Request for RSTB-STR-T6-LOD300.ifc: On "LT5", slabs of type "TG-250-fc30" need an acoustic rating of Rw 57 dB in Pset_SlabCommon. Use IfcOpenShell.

First a look at what the model holds.

```python
import ifcopenshell
import ifcopenshell.util.element

model = ifcopenshell.open("RSTB-STR-T6-LOD300.ifc")
print(model.schema)
storey = next(s for s in model.by_type("IfcBuildingStorey") if s.Name == "LT5")
slabs = [e for e in ifcopenshell.util.element.get_decomposition(storey) if e.is_a("IfcSlab")]
seen = {}
for e in slabs:
    element_type = ifcopenshell.util.element.get_type(e)
    key = (element_type.Name if element_type != e and element_type else None, ifcopenshell.util.element.get_pset(e, "Pset_SlabCommon", "AcousticRating"))
    seen[key] = seen.get(key, 0) + 1
for (name, value), count in sorted(seen.items(), key=str):
    print(count, "x", name, "|", value)
```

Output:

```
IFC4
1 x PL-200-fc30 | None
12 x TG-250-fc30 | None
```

```python
import ifcopenshell
import ifcopenshell.api.pset
import ifcopenshell.util.element

model = ifcopenshell.open("RSTB-STR-T6-LOD300.ifc")

storey = next(s for s in model.by_type("IfcBuildingStorey") if s.Name == "LT5")
slabs = [e for e in ifcopenshell.util.element.get_decomposition(storey) if e.is_a("IfcSlab")]

count = 0
for e in slabs:
    element_type = ifcopenshell.util.element.get_type(e)
    if element_type in (None, e) or element_type.Name != "TG-250-fc30":
        continue
    # add_pset returns the element's existing set when there is one.
    pset = ifcopenshell.api.pset.add_pset(model, product=e, name="Pset_SlabCommon")
    ifcopenshell.api.pset.edit_pset(model, pset=pset, properties={"AcousticRating": "Rw 57 dB"})
    count += 1

print(count, "slabs updated")

model.write("RSTB-STR-T6-LOD300_v2.ifc")
```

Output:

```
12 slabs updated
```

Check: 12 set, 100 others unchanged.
